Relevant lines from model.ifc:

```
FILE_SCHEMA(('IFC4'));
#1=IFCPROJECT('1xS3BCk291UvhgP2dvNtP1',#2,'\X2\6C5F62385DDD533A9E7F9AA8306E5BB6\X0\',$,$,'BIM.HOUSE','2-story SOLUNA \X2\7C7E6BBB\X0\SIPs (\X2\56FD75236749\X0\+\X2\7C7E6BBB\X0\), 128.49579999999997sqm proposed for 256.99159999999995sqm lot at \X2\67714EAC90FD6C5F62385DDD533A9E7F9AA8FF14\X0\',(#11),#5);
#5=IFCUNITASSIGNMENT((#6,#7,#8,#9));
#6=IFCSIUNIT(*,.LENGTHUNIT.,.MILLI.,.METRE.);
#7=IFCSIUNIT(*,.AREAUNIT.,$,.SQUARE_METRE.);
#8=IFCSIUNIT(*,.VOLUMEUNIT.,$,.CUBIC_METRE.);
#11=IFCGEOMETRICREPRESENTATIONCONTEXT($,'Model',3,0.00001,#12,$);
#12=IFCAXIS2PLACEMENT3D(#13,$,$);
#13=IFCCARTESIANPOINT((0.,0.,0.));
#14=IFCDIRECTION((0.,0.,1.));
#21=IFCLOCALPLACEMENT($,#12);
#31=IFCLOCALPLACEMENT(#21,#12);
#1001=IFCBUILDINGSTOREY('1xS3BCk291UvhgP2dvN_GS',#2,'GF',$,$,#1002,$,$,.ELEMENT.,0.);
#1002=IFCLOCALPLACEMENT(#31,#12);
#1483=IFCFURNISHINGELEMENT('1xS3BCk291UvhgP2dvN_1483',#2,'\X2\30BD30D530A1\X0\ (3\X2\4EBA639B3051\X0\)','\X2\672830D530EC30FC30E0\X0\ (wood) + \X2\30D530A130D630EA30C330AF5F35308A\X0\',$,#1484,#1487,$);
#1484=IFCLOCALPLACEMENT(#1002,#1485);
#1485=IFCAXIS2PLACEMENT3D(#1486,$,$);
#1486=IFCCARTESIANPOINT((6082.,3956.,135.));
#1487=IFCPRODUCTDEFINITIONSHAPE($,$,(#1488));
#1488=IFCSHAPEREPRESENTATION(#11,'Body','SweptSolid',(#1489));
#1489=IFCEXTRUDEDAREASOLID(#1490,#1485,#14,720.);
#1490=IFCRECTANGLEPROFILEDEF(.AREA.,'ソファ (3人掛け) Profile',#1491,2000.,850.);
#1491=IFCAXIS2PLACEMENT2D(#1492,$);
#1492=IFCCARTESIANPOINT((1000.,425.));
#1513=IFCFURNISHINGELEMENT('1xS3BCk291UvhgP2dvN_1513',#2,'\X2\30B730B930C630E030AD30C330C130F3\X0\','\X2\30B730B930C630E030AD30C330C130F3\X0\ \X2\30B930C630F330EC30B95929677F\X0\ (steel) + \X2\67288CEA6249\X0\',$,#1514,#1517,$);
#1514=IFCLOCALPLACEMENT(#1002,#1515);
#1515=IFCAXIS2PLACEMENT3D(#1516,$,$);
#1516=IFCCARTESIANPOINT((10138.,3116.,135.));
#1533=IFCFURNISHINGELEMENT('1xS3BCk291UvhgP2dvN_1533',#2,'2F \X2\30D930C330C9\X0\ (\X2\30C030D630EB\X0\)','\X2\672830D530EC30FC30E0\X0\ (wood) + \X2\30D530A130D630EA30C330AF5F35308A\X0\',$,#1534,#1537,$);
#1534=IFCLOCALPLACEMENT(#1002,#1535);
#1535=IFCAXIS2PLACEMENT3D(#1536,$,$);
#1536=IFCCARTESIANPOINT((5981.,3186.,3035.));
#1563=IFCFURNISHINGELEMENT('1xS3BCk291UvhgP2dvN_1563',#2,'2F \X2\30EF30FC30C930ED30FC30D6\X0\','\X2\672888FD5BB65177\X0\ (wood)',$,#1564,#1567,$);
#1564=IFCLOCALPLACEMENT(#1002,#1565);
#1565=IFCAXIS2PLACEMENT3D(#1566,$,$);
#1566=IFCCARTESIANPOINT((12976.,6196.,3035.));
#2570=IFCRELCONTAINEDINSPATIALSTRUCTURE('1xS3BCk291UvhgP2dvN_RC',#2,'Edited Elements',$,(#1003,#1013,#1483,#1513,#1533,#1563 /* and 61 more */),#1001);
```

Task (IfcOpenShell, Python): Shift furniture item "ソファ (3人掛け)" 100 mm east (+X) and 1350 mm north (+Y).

```python
import ifcopenshell
import ifcopenshell.api.geometry
import ifcopenshell.util.placement
import ifcopenshell.util.unit

model = ifcopenshell.open("model.ifc")
unit_scale = ifcopenshell.util.unit.calculate_unit_scale(model)

item = model.by_guid("1xS3BCk291UvhgP2dvN_1483")
matrix = ifcopenshell.util.placement.get_local_placement(item.ObjectPlacement)
matrix[0, 3] += 0.1 / unit_scale
matrix[1, 3] += 1.35 / unit_scale
ifcopenshell.api.geometry.edit_object_placement(model, product=item, matrix=matrix, is_si=False)

print(ifcopenshell.util.placement.get_local_placement(item.ObjectPlacement).round(3) + 0.0)

model.write("model_edited.ifc")
```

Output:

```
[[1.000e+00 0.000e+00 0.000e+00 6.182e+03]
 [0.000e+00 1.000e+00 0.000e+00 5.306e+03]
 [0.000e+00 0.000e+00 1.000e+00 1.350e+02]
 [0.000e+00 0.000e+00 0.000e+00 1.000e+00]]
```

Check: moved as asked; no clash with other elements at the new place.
